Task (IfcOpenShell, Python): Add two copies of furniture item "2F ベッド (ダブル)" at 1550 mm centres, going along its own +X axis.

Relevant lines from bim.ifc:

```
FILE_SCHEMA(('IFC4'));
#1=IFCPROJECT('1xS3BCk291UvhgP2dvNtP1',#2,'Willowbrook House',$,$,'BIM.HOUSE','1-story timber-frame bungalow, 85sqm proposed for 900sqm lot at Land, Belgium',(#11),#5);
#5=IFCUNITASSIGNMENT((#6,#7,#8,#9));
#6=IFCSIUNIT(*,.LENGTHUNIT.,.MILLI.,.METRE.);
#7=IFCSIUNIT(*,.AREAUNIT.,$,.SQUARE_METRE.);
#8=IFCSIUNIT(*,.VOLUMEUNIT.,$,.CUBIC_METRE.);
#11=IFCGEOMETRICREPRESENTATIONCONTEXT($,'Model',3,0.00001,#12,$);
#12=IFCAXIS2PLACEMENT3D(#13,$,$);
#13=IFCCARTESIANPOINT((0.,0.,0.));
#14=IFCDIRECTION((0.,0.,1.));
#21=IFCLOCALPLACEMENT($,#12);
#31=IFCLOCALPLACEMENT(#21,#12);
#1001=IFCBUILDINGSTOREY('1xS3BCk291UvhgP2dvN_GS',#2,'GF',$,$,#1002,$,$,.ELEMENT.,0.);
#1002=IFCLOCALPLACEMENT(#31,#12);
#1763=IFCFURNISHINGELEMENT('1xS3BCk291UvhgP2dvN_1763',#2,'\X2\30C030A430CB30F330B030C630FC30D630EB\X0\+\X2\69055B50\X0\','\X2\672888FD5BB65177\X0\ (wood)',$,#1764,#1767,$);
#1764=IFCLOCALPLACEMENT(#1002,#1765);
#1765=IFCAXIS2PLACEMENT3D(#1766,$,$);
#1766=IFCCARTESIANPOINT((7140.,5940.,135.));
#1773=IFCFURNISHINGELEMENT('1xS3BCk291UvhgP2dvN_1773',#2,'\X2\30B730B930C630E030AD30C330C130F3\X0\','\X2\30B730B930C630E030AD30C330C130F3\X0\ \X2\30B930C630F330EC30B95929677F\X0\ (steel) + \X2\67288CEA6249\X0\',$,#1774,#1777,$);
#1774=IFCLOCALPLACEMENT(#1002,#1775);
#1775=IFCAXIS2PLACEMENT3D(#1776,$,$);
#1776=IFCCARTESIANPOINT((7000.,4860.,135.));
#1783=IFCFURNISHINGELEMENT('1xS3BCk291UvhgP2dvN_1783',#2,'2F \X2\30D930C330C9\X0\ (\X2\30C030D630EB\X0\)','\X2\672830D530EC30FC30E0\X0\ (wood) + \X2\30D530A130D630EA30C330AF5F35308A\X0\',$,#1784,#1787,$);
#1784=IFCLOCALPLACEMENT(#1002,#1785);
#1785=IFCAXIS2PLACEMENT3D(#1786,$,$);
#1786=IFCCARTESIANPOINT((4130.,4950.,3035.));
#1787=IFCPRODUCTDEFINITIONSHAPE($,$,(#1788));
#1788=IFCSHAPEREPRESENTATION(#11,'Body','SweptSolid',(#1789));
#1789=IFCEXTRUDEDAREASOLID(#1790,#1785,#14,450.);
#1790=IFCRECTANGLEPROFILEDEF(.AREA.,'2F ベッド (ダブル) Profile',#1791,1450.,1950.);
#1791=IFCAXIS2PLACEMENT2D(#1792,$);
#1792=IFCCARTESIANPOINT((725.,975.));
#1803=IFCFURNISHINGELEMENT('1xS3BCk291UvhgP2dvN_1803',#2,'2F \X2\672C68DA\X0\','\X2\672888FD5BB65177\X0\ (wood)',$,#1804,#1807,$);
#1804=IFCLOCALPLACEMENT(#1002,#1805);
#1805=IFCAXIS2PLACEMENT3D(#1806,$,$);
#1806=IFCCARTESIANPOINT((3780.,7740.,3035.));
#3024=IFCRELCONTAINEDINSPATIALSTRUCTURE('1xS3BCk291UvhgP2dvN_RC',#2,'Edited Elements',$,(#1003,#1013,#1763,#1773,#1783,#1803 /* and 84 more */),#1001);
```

```python
import ifcopenshell
import ifcopenshell.api.geometry
import ifcopenshell.api.root
import ifcopenshell.util.element
import ifcopenshell.util.placement
import ifcopenshell.util.unit

model = ifcopenshell.open("bim.ifc")
unit_scale = ifcopenshell.util.unit.calculate_unit_scale(model)


def reuse_history(source, copy):
    """copy_class also copies each property set's owner history, people and application; keep the originals."""
    for rel in copy.IsDefinedBy:
        if rel.is_a("IfcRelDefinesByProperties") and (history := rel.RelatingPropertyDefinition.OwnerHistory):
            rel.RelatingPropertyDefinition.OwnerHistory = source.OwnerHistory
            ifcopenshell.util.element.remove_deep2(model, history)


source = model.by_guid("1xS3BCk291UvhgP2dvN_1783")
base = ifcopenshell.util.placement.get_local_placement(source.ObjectPlacement)
step = base[:3, 0] * 1.55 / unit_scale

for i in range(1, 3):
    copy = ifcopenshell.api.root.copy_class(model, product=source)
    copy.Representation = ifcopenshell.util.element.copy_deep(
        model, source.Representation, exclude=["IfcGeometricRepresentationContext", "IfcRepresentationMap"]
    )
    reuse_history(source, copy)
    matrix = base.copy()
    matrix[:3, 3] += i * step
    print("added at", matrix[:3, 3].round(3) + 0.0)
    ifcopenshell.api.geometry.edit_object_placement(model, product=copy, matrix=matrix, is_si=False)

model.write("bim_v2.ifc")
```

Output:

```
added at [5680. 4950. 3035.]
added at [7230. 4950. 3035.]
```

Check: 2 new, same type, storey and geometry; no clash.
